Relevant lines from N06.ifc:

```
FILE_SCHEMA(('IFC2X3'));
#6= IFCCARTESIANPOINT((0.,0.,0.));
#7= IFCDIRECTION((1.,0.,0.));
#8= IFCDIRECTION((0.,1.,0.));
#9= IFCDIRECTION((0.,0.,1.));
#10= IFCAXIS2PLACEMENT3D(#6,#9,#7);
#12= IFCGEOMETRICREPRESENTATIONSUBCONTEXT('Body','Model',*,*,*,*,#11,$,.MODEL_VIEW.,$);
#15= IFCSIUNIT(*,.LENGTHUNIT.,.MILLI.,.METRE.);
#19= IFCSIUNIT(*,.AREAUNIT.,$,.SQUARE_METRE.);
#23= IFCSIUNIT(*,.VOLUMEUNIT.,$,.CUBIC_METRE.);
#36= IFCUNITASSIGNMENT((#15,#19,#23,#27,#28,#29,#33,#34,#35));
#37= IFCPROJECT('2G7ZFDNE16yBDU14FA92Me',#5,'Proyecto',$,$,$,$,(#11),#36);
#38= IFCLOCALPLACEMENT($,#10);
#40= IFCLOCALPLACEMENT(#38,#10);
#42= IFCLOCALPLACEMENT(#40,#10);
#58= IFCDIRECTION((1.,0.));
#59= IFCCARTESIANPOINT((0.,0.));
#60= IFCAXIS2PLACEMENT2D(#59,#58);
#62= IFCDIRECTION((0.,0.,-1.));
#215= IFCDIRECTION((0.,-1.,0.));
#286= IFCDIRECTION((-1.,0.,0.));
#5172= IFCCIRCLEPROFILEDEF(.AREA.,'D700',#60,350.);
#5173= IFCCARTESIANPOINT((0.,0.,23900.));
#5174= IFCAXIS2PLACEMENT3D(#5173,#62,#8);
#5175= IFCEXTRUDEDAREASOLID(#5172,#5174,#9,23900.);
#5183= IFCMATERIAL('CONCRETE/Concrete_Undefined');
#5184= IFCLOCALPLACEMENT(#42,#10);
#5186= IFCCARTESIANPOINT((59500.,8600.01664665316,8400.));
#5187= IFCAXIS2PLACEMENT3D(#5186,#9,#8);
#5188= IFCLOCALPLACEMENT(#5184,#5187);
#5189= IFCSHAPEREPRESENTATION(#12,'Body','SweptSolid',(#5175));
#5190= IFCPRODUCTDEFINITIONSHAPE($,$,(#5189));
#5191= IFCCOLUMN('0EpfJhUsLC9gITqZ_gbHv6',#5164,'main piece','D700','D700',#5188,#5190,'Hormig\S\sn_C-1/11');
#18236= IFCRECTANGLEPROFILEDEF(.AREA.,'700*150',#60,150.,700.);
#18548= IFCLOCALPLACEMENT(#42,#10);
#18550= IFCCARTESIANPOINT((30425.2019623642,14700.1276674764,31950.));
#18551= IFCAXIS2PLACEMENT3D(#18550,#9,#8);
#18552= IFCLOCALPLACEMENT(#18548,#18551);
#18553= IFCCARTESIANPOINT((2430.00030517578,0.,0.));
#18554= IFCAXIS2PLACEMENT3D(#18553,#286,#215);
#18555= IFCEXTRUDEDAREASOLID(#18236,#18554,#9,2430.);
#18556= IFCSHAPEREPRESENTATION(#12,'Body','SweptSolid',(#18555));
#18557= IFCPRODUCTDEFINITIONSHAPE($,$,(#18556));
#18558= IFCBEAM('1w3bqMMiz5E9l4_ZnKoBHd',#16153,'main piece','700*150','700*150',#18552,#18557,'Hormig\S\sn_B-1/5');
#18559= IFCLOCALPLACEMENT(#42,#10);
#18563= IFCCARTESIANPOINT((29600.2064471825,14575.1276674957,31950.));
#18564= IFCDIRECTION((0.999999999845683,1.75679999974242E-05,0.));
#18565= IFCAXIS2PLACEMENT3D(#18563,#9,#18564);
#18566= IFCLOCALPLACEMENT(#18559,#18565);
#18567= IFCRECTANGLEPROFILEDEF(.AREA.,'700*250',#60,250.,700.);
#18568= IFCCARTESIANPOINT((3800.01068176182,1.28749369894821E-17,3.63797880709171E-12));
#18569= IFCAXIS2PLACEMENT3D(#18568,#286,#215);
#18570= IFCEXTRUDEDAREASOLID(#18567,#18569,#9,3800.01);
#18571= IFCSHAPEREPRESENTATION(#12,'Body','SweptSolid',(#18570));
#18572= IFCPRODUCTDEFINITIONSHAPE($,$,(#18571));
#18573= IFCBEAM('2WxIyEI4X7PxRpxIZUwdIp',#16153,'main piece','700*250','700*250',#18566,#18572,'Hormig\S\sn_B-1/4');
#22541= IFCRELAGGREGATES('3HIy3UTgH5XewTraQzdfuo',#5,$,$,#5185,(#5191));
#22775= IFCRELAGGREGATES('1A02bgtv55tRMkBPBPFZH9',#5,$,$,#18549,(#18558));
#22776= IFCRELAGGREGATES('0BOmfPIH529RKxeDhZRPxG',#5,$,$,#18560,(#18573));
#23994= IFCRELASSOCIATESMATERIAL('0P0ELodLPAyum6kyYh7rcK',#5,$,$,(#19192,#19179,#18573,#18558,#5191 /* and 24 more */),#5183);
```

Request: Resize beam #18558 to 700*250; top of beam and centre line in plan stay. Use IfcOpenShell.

```python
import ifcopenshell
import ifcopenshell.util.element
import ifcopenshell.util.representation

model = ifcopenshell.open("N06.ifc")

member = model.by_id(18558)
source = next(p for p in model.by_type("IfcRectangleProfileDef") if p.ProfileName == "700*250")

body = ifcopenshell.util.representation.get_representation(member, "Model", "Body")
solid = body.Items[0]
old_profile = solid.SweptArea

# Copy the section's sizes but keep this member's own profile position.
profile = ifcopenshell.util.element.copy(model, source)
# Profiles are centred, so shift by half the change in depth to hold the top.
shift = (old_profile.YDim - profile.YDim) / 2
x, y = old_profile.Position.Location.Coordinates
up = (0.0, 1.0)  # upwards, in the solid's own plane
location = model.createIfcCartesianPoint((x + up[0] * shift, y + up[1] * shift))
profile.Position = model.createIfcAxis2Placement2D(location, old_profile.Position.RefDirection)
solid.SweptArea = profile
if not model.get_total_inverses(old_profile):
    ifcopenshell.util.element.remove_deep2(model, old_profile)
member.Description = member.Description.replace("700*150", "700*250")
member.ObjectType = member.ObjectType.replace("700*150", "700*250")

print(solid.SweptArea)

model.write("N06_edited.ifc")
```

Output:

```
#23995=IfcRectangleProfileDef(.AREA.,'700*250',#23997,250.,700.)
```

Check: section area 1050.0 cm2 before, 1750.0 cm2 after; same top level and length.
